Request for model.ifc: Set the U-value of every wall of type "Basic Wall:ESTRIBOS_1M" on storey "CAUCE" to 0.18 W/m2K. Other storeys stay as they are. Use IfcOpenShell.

First a look at what the model holds.

```python
import ifcopenshell
import ifcopenshell.util.element

model = ifcopenshell.open("model.ifc")
print(model.schema)
storey = next(s for s in model.by_type("IfcBuildingStorey") if s.Name == "CAUCE")
walls = [e for e in ifcopenshell.util.element.get_decomposition(storey) if e.is_a("IfcWall")]
seen = {}
for e in walls:
    element_type = ifcopenshell.util.element.get_type(e)
    key = (element_type.Name if element_type != e and element_type else None, ifcopenshell.util.element.get_pset(e, "Pset_WallCommon", "ThermalTransmittance"))
    seen[key] = seen.get(key, 0) + 1
for (name, value), count in sorted(seen.items(), key=str):
    print(count, "x", name, "|", value)
```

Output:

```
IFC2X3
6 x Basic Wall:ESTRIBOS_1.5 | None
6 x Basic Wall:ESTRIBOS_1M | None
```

```python
import ifcopenshell
import ifcopenshell.api.pset
import ifcopenshell.util.element

model = ifcopenshell.open("model.ifc")

storey = next(s for s in model.by_type("IfcBuildingStorey") if s.Name == "CAUCE")
walls = [e for e in ifcopenshell.util.element.get_decomposition(storey) if e.is_a("IfcWall")]

count = 0
for e in walls:
    element_type = ifcopenshell.util.element.get_type(e)
    if element_type in (None, e) or element_type.Name != "Basic Wall:ESTRIBOS_1M":
        continue
    # add_pset returns the element's existing set when there is one.
    pset = ifcopenshell.api.pset.add_pset(model, product=e, name="Pset_WallCommon")
    ifcopenshell.api.pset.edit_pset(model, pset=pset, properties={"ThermalTransmittance": 0.18})
    count += 1

print(count, "walls updated")

model.write("model_edited.ifc")
```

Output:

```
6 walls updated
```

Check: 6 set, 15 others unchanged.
